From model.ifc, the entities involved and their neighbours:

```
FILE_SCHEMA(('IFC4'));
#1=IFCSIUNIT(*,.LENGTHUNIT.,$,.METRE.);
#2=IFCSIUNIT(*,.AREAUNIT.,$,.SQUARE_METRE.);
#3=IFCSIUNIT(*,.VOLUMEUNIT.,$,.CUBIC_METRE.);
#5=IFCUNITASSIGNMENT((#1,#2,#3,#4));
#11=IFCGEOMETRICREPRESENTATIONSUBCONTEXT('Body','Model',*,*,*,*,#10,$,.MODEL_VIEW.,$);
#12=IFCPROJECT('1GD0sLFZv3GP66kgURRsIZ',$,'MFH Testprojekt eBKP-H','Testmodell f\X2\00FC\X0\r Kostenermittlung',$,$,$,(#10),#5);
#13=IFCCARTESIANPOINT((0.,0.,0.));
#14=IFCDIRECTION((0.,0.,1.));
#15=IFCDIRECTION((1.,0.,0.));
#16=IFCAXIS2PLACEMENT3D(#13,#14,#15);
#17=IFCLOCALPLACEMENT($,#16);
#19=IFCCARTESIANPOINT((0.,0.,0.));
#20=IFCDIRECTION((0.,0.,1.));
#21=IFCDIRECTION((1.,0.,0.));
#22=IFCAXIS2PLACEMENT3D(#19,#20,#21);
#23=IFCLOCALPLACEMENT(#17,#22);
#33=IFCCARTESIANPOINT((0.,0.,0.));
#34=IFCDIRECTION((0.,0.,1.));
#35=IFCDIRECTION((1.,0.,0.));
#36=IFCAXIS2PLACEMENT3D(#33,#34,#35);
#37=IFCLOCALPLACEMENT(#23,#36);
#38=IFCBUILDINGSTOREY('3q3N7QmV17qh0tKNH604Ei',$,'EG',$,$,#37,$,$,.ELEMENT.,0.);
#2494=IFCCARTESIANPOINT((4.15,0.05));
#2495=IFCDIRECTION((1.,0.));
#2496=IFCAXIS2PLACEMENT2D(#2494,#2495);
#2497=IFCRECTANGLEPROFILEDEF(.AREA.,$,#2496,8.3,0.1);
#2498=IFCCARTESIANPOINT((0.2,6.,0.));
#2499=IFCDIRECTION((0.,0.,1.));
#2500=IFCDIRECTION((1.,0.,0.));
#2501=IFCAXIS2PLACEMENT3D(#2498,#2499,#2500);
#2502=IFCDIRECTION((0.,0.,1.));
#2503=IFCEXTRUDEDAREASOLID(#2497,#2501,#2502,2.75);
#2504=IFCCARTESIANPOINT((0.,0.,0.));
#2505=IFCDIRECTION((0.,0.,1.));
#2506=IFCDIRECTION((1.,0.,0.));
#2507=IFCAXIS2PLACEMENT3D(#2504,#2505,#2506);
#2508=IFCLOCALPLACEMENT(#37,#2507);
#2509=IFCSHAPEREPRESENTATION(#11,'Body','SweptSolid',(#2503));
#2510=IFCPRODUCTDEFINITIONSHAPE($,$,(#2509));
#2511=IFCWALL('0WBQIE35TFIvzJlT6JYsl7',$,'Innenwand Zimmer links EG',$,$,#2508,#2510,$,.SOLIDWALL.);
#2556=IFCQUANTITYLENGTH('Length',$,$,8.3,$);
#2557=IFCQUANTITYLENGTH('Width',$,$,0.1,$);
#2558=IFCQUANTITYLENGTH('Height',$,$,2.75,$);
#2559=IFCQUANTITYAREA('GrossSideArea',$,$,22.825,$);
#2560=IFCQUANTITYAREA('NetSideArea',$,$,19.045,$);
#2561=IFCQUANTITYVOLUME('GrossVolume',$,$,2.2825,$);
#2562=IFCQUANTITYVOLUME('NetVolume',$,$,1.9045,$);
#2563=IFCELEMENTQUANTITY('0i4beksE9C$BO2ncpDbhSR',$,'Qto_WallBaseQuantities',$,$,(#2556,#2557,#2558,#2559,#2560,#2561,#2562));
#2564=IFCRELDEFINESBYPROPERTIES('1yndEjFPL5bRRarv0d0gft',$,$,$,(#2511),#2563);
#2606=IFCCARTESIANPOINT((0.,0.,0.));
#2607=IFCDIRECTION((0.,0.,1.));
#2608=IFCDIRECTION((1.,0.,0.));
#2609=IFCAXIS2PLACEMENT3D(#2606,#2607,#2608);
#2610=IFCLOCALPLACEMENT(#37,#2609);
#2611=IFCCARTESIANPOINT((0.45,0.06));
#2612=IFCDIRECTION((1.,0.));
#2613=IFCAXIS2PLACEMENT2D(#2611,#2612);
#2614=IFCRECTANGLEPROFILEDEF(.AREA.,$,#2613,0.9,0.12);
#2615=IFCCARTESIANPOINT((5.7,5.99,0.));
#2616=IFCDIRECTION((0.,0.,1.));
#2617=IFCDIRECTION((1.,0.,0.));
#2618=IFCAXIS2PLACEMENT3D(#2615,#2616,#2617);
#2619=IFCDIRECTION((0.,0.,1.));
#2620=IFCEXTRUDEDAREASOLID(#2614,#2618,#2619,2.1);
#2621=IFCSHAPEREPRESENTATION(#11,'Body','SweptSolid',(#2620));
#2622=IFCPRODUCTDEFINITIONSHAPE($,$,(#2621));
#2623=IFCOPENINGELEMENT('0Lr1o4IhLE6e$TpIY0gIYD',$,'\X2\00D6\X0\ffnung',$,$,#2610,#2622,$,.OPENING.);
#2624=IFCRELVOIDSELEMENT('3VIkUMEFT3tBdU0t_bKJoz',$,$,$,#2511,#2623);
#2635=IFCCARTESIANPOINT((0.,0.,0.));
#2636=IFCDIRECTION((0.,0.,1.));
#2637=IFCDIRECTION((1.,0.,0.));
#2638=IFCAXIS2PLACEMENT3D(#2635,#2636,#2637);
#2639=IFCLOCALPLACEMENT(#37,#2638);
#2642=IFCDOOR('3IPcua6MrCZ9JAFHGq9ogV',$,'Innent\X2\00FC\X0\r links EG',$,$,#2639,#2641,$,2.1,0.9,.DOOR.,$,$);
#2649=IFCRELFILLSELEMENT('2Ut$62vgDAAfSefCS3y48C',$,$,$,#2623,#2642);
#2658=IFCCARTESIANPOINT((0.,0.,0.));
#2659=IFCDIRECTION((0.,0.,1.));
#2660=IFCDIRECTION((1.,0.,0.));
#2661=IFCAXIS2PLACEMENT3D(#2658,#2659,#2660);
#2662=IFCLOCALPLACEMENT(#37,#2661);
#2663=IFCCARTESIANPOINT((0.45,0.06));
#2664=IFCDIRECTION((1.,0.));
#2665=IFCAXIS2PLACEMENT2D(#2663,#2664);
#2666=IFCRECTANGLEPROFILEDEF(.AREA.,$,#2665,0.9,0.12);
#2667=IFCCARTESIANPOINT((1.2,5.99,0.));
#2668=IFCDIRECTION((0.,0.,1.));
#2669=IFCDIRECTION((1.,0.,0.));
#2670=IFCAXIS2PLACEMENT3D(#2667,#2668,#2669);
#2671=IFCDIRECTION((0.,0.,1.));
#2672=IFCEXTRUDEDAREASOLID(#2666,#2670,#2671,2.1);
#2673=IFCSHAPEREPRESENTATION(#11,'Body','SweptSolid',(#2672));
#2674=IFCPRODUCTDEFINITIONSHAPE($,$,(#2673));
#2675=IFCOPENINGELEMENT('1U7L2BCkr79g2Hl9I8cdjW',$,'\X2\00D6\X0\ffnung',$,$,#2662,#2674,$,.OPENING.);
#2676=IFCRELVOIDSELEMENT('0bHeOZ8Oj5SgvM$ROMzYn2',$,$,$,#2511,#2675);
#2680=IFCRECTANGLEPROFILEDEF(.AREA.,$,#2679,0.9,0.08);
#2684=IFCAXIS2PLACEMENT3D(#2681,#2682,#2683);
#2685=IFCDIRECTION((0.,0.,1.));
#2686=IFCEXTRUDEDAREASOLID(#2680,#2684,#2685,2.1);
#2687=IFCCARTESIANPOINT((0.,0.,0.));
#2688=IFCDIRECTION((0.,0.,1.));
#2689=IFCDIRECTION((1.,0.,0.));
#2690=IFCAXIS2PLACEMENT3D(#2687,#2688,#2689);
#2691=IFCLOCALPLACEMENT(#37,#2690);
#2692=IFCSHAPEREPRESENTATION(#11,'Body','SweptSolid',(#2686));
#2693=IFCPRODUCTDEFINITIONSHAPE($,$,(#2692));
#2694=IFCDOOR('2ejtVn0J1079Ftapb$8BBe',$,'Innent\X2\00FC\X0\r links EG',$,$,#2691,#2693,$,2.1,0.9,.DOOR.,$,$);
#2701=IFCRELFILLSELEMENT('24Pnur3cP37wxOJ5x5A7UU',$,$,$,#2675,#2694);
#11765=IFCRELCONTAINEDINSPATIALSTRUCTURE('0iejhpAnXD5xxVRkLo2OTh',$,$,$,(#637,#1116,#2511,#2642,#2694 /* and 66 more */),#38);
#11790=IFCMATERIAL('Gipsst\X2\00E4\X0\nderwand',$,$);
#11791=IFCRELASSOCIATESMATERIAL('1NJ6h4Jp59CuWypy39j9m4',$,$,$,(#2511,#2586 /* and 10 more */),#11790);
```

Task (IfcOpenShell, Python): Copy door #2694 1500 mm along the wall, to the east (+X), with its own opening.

```python
import ifcopenshell
import ifcopenshell.api.feature
import ifcopenshell.api.geometry
import ifcopenshell.api.pset
import ifcopenshell.api.root
import ifcopenshell.geom
import ifcopenshell.util.element
import ifcopenshell.util.placement
import ifcopenshell.util.shape
import ifcopenshell.util.unit

model = ifcopenshell.open("model.ifc")
unit_scale = ifcopenshell.util.unit.calculate_unit_scale(model)
area_scale = ifcopenshell.util.unit.calculate_unit_scale(model, "AREAUNIT")
volume_scale = ifcopenshell.util.unit.calculate_unit_scale(model, "VOLUMEUNIT")
settings = ifcopenshell.geom.settings()


def volume(element):
    """Net volume in cubic metres, openings subtracted."""
    shape = ifcopenshell.geom.create_shape(settings, element)
    return ifcopenshell.util.shape.get_volume(shape.geometry)


door = model.by_guid("2ejtVn0J1079Ftapb$8BBe")
opening = door.FillsVoids[0].RelatingOpeningElement
wall = opening.VoidsElements[0].RelatingBuildingElement
before = volume(wall)
shift = ifcopenshell.util.placement.get_local_placement(wall.ObjectPlacement)[:3, 0] * 1.5 / unit_scale

# copy_class copies the void relationship, type, container and properties, but no geometry.
new_opening = ifcopenshell.api.root.copy_class(model, product=opening)
new_opening.Representation = ifcopenshell.util.element.copy_deep(
    model, opening.Representation, exclude=["IfcGeometricRepresentationContext", "IfcRepresentationMap"]
)
new_door = ifcopenshell.api.root.copy_class(model, product=door)
new_door.Representation = ifcopenshell.util.element.copy_deep(
    model, door.Representation, exclude=["IfcGeometricRepresentationContext", "IfcRepresentationMap"]
)
ifcopenshell.api.feature.add_filling(model, opening=new_opening, element=new_door)

for old, new in ((opening, new_opening), (door, new_door)):
    matrix = ifcopenshell.util.placement.get_local_placement(old.ObjectPlacement)
    matrix[:3, 3] += shift
    ifcopenshell.api.geometry.edit_object_placement(model, product=new, matrix=matrix, is_si=False)

after = volume(wall)
thickness = 0.1  # wall thickness in metres

# Update the wall's stored quantities.
qto = model.by_id(ifcopenshell.util.element.get_pset(wall, "Qto_WallBaseQuantities", should_inherit=False)["id"])
ifcopenshell.api.pset.edit_qto(model, qto=qto, properties={
    "NetSideArea": after / thickness / area_scale,
    "NetVolume": after / volume_scale,
})

print(f"wall volume {before:.3f} -> {after:.3f} m3")

model.write("model_edited.ifc")
```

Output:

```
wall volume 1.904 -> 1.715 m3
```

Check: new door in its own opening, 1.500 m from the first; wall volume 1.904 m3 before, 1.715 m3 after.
